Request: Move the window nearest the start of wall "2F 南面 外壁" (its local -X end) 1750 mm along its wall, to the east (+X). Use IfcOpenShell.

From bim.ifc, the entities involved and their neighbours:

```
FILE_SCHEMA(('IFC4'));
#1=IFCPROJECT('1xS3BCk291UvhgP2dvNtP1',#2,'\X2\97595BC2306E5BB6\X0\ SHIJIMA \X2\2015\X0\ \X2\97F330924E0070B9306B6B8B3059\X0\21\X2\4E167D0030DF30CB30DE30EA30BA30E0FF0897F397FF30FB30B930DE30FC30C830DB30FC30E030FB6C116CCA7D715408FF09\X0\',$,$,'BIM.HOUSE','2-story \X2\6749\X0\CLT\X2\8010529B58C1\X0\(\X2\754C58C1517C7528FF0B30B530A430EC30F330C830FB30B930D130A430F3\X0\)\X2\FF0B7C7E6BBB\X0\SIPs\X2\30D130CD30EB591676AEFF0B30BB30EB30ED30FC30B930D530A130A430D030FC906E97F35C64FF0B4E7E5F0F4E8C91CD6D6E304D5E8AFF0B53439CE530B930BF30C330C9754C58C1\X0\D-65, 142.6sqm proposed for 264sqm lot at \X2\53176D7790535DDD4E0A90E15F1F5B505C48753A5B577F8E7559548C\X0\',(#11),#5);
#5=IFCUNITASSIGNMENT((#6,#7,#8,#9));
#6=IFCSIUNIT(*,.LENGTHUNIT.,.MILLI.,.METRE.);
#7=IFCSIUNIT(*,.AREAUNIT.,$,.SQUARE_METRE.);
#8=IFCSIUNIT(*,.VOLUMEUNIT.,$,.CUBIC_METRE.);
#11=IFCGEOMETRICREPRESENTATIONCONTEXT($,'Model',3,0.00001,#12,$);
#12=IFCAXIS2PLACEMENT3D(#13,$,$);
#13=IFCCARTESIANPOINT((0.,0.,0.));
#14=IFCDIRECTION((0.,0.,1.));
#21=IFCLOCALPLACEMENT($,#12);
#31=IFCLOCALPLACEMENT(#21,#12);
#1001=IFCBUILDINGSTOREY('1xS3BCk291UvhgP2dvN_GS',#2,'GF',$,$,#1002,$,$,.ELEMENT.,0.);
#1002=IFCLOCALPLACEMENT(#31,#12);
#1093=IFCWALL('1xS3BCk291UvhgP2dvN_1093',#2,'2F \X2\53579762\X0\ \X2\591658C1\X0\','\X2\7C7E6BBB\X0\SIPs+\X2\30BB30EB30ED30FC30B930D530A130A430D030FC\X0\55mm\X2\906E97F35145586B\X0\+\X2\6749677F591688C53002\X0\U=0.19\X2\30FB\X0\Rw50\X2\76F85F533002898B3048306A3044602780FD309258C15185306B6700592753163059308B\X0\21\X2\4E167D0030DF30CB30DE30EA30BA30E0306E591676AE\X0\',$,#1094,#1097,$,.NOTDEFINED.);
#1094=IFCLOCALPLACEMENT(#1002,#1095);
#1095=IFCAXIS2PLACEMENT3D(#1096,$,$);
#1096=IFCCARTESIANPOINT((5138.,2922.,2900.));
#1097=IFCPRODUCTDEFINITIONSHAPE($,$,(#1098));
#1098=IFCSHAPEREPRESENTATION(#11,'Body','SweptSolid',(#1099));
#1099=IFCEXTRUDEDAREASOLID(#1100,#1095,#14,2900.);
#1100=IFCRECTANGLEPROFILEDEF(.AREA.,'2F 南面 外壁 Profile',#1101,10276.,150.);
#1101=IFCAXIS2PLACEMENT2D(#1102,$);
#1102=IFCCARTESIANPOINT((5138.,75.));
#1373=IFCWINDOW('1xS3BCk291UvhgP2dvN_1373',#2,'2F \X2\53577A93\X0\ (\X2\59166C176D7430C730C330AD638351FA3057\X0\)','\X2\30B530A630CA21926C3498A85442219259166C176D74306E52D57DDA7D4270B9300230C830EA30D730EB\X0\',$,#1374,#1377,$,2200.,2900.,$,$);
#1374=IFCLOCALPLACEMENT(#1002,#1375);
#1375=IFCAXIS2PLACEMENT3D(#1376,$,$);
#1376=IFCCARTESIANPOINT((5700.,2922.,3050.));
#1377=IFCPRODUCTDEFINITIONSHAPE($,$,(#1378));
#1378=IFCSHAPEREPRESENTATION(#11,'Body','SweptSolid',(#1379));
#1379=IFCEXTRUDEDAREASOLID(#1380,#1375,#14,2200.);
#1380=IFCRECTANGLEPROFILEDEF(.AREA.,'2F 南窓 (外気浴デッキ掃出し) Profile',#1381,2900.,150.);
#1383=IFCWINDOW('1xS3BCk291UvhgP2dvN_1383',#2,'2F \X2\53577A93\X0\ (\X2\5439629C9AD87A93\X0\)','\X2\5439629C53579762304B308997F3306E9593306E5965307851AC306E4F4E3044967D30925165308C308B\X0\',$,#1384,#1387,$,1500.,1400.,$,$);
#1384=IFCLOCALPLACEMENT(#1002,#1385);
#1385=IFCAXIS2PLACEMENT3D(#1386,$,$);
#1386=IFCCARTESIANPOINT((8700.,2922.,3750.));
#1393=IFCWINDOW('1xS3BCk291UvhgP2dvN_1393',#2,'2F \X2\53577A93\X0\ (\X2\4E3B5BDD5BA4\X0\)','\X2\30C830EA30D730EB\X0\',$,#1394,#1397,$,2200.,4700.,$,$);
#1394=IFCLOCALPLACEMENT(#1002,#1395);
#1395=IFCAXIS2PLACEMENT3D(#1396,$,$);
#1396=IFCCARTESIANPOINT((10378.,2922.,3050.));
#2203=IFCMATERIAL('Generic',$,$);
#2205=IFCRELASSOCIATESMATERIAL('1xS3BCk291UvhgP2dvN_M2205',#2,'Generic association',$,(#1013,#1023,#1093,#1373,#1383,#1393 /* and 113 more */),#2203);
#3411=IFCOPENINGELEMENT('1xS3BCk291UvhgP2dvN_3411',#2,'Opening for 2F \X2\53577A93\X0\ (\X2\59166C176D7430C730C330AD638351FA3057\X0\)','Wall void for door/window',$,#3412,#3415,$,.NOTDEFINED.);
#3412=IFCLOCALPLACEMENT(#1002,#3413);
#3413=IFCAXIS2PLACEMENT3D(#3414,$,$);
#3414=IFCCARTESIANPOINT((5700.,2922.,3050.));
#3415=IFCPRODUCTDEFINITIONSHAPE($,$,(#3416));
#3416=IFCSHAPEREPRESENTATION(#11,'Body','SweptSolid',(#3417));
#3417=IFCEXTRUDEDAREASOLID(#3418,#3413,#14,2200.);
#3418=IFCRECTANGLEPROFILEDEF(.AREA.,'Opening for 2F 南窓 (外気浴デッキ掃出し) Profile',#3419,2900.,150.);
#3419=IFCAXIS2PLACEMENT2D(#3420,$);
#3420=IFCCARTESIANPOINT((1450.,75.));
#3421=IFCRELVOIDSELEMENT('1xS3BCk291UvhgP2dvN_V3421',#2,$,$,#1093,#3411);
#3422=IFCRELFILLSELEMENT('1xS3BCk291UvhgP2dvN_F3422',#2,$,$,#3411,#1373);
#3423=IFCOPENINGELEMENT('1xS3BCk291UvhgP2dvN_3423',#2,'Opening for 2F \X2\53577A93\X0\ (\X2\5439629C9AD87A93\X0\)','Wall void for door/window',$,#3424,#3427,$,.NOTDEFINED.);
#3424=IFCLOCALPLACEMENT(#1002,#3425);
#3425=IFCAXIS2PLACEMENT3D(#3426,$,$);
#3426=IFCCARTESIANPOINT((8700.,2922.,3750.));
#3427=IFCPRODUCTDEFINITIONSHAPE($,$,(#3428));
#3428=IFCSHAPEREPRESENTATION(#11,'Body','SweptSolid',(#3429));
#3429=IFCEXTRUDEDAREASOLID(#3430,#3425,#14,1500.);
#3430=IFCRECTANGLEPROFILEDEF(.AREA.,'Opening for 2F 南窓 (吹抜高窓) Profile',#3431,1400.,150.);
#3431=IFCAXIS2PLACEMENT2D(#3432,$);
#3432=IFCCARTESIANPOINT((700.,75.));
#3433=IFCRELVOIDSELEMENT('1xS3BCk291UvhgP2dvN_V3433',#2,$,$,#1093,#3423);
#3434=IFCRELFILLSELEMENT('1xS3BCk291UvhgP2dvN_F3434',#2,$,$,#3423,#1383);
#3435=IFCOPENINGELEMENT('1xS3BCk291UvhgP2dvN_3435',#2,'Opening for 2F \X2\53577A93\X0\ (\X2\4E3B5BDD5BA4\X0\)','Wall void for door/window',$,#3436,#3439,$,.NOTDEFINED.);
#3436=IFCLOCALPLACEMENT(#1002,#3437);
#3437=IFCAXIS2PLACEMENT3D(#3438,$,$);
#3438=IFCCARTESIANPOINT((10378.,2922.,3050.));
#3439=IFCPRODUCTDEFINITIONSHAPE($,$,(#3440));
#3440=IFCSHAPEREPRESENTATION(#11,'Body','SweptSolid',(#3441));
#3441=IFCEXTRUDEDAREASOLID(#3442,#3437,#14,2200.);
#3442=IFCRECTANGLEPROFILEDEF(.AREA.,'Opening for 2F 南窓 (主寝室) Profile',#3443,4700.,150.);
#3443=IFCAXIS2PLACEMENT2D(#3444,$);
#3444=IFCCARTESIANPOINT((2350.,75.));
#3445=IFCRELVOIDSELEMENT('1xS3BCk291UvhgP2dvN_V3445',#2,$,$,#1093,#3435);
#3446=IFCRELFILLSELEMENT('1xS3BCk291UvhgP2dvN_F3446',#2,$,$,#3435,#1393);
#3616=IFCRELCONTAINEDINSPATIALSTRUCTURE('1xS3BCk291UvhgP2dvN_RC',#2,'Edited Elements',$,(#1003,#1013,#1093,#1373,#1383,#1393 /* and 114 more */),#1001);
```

```python
import ifcopenshell
import ifcopenshell.api.geometry
import ifcopenshell.util.placement

model = ifcopenshell.open("bim.ifc")

window = model.by_guid("1xS3BCk291UvhgP2dvN_1373")
opening = window.FillsVoids[0].RelatingOpeningElement
wall = opening.VoidsElements[0].RelatingBuildingElement

wall_matrix = ifcopenshell.util.placement.get_local_placement(wall.ObjectPlacement)
shift = wall_matrix[:3, 0] * 1750.0
before = ifcopenshell.util.placement.get_local_placement(window.ObjectPlacement)[:3, 3].copy()

# The window is not placed relative to its opening, so move both.
for product in (opening, window):
    matrix = ifcopenshell.util.placement.get_local_placement(product.ObjectPlacement)
    matrix[:3, 3] += shift
    ifcopenshell.api.geometry.edit_object_placement(model, product=product, matrix=matrix, is_si=False)

after = ifcopenshell.util.placement.get_local_placement(window.ObjectPlacement)[:3, 3]
print("window moved by", (after - before).round(3) + 0.0)

model.write("bim_v2.ifc")
```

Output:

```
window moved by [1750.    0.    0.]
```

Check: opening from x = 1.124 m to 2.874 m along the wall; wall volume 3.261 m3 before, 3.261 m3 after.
